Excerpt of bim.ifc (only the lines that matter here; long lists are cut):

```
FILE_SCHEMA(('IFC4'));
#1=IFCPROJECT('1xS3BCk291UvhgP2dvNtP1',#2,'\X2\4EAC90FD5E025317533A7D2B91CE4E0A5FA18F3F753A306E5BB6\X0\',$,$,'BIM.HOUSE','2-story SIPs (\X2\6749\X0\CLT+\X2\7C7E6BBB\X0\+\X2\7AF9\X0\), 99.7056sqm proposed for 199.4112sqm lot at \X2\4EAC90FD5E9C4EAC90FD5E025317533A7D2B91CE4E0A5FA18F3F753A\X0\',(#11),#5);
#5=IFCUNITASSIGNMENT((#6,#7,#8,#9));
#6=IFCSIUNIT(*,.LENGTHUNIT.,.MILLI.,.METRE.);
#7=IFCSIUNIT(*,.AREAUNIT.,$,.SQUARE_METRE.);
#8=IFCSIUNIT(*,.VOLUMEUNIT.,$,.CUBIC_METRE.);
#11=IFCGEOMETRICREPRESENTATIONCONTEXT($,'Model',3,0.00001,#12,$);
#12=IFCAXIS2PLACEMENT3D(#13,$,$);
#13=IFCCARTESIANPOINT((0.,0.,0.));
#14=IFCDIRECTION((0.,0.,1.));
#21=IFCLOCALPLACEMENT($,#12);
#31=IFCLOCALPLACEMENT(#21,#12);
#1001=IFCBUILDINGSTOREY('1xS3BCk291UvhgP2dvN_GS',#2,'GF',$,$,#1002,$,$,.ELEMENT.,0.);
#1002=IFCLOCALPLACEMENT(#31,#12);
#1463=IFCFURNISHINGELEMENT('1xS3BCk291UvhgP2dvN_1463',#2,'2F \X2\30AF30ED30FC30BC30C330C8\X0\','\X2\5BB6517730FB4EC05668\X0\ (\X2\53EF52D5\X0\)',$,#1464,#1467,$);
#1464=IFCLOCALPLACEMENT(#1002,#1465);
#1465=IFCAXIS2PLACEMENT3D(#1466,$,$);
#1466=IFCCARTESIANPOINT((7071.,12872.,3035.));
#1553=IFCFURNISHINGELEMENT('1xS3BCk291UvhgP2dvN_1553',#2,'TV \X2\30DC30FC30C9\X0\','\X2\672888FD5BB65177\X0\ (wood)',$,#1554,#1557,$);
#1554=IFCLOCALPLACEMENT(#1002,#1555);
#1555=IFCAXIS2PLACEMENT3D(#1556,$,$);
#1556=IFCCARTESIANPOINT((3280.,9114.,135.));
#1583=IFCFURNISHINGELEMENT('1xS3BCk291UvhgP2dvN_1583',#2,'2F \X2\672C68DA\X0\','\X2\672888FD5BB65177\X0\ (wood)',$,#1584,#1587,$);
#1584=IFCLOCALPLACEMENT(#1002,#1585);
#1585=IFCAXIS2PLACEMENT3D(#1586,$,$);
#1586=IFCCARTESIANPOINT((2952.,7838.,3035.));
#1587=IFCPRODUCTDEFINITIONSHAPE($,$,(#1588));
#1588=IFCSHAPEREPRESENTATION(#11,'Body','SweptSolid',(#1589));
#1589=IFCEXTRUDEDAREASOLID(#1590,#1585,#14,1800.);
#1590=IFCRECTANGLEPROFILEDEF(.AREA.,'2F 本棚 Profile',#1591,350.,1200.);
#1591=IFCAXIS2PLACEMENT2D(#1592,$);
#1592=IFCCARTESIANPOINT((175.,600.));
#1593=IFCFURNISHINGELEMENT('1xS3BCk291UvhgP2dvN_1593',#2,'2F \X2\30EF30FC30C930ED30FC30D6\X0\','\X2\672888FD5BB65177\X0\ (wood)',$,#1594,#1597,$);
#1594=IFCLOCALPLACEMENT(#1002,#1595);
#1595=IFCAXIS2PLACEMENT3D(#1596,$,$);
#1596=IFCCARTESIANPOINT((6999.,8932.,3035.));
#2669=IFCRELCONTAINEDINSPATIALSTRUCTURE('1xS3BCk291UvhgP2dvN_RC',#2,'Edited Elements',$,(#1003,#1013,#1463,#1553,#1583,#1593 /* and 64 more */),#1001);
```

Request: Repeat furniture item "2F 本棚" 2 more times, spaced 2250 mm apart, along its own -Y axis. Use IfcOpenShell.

```python
import ifcopenshell
import ifcopenshell.api.geometry
import ifcopenshell.api.root
import ifcopenshell.util.element
import ifcopenshell.util.placement
import ifcopenshell.util.unit

model = ifcopenshell.open("bim.ifc")
unit_scale = ifcopenshell.util.unit.calculate_unit_scale(model)


def reuse_history(source, copy):
    """copy_class also copies each property set's owner history, people and application; keep the originals."""
    for rel in copy.IsDefinedBy:
        if rel.is_a("IfcRelDefinesByProperties") and (history := rel.RelatingPropertyDefinition.OwnerHistory):
            rel.RelatingPropertyDefinition.OwnerHistory = source.OwnerHistory
            ifcopenshell.util.element.remove_deep2(model, history)


source = model.by_guid("1xS3BCk291UvhgP2dvN_1583")
base = ifcopenshell.util.placement.get_local_placement(source.ObjectPlacement)
step = -base[:3, 1] * 2.25 / unit_scale

for i in range(1, 3):
    copy = ifcopenshell.api.root.copy_class(model, product=source)
    copy.Representation = ifcopenshell.util.element.copy_deep(
        model, source.Representation, exclude=["IfcGeometricRepresentationContext", "IfcRepresentationMap"]
    )
    reuse_history(source, copy)
    matrix = base.copy()
    matrix[:3, 3] += i * step
    print("added at", matrix[:3, 3].round(3) + 0.0)
    ifcopenshell.api.geometry.edit_object_placement(model, product=copy, matrix=matrix, is_si=False)

model.write("bim_edited.ifc")
```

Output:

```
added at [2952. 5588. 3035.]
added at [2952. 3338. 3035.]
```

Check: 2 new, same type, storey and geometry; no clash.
